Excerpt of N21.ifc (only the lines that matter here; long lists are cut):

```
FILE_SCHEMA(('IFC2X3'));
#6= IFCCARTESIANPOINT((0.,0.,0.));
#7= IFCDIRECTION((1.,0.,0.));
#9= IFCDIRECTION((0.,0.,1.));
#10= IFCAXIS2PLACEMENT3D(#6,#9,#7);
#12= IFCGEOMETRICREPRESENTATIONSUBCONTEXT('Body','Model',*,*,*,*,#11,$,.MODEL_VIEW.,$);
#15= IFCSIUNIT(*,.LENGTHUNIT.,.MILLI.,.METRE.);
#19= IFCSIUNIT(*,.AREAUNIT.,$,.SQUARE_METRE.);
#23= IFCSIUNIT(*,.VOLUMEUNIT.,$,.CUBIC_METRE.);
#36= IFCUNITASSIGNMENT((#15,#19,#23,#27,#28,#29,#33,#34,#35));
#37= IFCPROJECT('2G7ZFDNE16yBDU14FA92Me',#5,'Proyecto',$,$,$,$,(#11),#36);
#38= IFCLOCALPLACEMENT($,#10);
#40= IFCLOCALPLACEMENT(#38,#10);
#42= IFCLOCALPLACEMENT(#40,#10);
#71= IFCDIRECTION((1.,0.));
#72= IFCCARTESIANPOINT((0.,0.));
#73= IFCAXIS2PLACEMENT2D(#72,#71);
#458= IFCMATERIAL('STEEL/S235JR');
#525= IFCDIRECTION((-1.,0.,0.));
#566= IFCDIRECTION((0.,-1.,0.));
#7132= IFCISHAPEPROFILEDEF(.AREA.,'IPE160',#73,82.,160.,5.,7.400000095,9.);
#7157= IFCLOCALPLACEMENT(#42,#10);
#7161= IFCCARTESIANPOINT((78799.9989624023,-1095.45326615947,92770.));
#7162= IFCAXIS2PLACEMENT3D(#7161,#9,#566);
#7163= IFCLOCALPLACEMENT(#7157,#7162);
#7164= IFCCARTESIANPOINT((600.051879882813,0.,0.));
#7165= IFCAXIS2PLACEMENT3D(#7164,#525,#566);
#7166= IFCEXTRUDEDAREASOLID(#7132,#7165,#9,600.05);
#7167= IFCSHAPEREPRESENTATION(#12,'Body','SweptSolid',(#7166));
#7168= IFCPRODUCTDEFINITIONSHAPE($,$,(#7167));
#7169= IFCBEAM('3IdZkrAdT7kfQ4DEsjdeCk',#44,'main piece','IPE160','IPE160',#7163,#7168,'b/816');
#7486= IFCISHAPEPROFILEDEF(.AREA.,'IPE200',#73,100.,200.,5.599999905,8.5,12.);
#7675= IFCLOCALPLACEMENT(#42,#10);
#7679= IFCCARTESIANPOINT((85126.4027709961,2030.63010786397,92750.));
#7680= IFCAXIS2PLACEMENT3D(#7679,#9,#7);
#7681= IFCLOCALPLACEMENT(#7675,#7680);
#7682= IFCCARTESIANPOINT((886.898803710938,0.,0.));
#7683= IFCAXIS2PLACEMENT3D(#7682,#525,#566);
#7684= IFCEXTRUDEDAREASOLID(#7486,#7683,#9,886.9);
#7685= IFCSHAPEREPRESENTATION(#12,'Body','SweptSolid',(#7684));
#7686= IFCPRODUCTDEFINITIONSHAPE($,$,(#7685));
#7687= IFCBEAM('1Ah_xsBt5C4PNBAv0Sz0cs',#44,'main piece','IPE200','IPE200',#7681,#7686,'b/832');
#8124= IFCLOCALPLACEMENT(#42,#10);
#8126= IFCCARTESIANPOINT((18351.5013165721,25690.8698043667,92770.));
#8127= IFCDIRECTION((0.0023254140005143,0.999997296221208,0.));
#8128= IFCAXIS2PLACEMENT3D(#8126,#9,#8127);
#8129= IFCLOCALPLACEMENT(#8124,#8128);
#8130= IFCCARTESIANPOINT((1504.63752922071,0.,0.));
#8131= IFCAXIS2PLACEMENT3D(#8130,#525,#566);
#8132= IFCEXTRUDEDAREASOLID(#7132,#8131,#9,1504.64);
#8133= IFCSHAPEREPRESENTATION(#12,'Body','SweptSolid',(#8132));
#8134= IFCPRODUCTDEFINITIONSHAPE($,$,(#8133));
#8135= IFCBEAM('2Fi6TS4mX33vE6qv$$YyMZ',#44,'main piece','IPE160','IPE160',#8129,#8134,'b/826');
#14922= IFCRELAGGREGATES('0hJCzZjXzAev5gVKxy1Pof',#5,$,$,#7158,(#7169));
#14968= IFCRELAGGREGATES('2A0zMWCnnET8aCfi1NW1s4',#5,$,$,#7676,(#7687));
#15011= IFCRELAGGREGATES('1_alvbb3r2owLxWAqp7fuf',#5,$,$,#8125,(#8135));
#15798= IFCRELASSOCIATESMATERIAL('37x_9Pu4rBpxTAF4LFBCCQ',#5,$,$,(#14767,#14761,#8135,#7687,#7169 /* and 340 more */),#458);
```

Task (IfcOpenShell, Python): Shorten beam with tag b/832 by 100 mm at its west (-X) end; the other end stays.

```python
import ifcopenshell
import ifcopenshell.util.representation
import ifcopenshell.util.unit

model = ifcopenshell.open("N21.ifc")
unit_scale = ifcopenshell.util.unit.calculate_unit_scale(model)

member = model.by_guid("1Ah_xsBt5C4PNBAv0Sz0cs")
change = -0.1 / unit_scale

# The extrusion runs towards the end named, so only its depth changes.
body = ifcopenshell.util.representation.get_representation(member, "Model", "Body")
solid = body.Items[0]
old_length = solid.Depth
solid.Depth += change

print(f"length {old_length:g} -> {solid.Depth:g}")

model.write("N21_v2.ifc")
```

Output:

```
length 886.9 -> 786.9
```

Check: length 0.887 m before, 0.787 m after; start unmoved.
